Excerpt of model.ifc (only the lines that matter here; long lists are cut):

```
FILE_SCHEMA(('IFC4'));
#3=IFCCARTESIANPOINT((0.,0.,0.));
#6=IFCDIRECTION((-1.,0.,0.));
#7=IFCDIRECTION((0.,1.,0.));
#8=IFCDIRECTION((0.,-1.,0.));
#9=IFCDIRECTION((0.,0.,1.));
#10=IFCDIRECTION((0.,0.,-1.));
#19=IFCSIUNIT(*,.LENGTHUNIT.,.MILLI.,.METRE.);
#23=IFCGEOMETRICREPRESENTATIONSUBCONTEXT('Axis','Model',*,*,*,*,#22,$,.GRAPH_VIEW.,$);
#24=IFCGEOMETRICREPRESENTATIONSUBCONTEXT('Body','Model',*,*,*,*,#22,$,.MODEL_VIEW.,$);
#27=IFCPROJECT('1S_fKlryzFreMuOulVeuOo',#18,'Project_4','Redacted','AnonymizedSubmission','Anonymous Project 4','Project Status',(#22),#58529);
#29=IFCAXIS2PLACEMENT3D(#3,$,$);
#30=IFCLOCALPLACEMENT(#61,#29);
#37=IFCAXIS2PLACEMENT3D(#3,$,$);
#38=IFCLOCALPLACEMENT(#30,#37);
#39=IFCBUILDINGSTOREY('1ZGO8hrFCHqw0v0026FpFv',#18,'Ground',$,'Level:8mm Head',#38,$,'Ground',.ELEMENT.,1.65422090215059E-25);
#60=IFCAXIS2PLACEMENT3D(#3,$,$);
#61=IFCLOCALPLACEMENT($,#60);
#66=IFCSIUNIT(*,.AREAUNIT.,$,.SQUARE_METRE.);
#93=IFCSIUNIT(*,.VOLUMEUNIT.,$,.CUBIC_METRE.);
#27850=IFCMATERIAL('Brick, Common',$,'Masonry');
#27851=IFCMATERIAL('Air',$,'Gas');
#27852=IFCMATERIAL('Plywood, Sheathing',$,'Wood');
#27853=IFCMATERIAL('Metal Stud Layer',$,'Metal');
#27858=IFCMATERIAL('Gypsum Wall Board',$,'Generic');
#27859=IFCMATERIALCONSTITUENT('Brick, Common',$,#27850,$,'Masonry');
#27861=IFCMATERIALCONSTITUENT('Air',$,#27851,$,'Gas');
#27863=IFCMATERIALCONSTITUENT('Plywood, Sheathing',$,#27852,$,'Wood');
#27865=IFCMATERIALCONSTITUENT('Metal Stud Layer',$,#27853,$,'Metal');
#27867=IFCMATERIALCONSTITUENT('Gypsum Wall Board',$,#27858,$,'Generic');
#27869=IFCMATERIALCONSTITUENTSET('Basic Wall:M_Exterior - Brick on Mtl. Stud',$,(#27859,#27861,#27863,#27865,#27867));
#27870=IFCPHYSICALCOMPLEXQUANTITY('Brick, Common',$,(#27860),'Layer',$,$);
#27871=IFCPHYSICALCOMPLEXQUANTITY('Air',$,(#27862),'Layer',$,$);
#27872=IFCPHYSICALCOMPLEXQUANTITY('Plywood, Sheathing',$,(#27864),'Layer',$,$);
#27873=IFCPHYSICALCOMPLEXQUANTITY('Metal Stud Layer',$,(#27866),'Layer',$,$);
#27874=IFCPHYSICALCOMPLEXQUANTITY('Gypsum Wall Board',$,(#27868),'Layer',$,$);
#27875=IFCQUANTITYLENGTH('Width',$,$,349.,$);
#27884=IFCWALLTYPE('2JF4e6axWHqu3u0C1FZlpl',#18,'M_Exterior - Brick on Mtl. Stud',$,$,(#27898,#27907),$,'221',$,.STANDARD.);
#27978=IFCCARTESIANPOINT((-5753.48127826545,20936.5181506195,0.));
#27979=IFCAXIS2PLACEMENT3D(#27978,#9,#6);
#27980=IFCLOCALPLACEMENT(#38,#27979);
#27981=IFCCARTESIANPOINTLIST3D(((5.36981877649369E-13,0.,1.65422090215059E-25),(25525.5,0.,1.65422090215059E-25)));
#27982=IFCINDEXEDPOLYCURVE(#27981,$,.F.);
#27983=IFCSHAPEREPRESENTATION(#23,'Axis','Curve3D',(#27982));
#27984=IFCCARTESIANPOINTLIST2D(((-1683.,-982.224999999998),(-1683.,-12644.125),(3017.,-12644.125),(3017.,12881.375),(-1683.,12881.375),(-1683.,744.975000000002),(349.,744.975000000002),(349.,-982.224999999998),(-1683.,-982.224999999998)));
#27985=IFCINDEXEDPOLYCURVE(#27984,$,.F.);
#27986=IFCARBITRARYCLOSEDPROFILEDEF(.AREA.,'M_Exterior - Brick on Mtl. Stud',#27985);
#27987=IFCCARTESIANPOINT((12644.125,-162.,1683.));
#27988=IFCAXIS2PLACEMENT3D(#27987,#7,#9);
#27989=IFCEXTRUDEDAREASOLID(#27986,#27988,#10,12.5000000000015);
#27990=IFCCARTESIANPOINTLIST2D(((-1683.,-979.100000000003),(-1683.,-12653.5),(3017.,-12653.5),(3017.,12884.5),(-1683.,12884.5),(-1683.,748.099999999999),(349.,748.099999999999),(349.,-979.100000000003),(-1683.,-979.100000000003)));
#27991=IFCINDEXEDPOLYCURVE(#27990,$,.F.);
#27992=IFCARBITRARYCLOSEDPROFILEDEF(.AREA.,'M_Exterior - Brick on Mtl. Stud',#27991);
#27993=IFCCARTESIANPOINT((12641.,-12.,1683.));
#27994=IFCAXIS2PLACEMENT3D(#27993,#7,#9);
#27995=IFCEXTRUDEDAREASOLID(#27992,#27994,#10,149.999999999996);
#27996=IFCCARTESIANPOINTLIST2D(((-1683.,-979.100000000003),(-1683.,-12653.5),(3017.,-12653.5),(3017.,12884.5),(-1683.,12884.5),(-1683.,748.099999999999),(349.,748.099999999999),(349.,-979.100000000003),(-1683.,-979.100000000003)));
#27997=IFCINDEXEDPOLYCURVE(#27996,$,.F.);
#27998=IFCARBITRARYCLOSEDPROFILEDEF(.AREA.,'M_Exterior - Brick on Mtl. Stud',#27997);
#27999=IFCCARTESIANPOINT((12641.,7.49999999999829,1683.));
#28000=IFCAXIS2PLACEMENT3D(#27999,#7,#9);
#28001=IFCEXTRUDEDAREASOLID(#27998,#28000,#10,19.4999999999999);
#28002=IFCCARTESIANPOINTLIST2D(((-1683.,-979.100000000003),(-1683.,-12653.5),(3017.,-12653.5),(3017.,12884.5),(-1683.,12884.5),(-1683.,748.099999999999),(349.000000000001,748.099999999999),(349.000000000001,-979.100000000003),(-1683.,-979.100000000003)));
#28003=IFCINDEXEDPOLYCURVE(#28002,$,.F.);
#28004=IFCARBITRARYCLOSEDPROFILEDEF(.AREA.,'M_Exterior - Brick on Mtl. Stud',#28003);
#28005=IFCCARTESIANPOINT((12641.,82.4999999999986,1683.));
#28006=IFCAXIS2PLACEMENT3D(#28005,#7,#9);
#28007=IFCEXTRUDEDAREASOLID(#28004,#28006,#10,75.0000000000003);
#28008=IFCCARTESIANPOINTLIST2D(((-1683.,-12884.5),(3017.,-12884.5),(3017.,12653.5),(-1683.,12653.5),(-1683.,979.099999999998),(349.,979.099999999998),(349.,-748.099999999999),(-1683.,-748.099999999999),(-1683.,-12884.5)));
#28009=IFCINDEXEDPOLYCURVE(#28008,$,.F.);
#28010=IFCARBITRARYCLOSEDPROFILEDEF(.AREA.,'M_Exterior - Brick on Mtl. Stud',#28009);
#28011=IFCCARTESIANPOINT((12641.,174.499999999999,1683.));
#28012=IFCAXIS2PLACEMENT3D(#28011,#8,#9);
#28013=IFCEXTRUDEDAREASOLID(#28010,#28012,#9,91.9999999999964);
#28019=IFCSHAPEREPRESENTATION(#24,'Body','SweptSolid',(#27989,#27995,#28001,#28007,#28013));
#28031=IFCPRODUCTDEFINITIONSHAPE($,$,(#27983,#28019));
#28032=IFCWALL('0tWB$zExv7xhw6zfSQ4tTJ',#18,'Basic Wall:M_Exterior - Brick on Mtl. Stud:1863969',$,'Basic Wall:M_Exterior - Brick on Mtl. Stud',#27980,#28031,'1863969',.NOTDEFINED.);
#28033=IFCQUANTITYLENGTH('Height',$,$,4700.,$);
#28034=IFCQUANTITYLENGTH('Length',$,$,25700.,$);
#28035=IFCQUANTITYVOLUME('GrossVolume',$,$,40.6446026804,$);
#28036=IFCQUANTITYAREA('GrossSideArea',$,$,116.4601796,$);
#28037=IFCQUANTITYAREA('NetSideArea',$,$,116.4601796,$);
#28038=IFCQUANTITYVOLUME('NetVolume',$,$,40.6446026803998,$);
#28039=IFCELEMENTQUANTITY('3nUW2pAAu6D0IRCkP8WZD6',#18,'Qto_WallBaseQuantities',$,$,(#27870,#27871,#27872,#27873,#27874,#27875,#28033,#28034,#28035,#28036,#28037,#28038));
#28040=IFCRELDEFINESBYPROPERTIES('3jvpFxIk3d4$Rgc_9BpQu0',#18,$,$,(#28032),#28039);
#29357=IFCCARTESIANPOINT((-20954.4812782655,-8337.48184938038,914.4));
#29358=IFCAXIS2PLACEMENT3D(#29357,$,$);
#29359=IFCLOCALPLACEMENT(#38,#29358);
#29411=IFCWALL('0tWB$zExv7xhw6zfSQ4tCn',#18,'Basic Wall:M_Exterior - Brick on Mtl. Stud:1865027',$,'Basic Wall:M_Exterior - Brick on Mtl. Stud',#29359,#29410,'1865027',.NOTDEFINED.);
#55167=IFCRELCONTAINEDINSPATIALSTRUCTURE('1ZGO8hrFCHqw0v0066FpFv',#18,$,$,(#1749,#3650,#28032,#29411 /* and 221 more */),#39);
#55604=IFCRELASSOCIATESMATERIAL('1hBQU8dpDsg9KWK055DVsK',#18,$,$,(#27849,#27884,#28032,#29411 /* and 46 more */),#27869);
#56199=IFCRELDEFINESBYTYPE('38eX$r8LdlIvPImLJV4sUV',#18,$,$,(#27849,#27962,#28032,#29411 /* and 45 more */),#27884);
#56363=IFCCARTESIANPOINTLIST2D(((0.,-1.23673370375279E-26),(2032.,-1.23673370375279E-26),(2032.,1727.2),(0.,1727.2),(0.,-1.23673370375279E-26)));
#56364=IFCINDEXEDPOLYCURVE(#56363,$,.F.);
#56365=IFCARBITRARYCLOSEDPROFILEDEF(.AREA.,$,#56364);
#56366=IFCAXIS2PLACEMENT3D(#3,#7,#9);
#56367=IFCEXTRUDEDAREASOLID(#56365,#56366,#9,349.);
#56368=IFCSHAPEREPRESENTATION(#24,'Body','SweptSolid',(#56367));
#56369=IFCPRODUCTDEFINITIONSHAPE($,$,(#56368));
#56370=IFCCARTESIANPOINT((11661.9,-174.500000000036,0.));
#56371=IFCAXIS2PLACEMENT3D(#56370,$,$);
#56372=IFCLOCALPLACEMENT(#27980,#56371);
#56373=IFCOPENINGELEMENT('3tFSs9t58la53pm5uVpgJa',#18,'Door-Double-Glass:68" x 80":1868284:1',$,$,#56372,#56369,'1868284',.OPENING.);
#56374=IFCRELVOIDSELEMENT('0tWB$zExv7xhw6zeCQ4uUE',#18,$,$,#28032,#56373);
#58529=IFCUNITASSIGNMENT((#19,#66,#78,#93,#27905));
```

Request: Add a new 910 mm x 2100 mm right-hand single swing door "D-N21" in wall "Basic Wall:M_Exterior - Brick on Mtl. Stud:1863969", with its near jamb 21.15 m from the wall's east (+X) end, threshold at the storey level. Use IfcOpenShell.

```python
import numpy as np
import ifcopenshell
import ifcopenshell.api.feature
import ifcopenshell.api.geometry
import ifcopenshell.api.pset
import ifcopenshell.api.root
import ifcopenshell.api.spatial
import ifcopenshell.geom
import ifcopenshell.util.element
import ifcopenshell.util.placement
import ifcopenshell.util.representation
import ifcopenshell.util.shape
import ifcopenshell.util.unit

model = ifcopenshell.open("model.ifc")
unit_scale = ifcopenshell.util.unit.calculate_unit_scale(model)
area_scale = ifcopenshell.util.unit.calculate_unit_scale(model, "AREAUNIT")
volume_scale = ifcopenshell.util.unit.calculate_unit_scale(model, "VOLUMEUNIT")
settings = ifcopenshell.geom.settings()


def volume(element):
    """Net volume in cubic metres, openings subtracted."""
    shape = ifcopenshell.geom.create_shape(settings, element)
    return ifcopenshell.util.shape.get_volume(shape.geometry)


wall = model.by_id(28032)
storey = ifcopenshell.util.element.get_container(wall, ifc_class="IfcBuildingStorey")
context = ifcopenshell.util.representation.get_context(model, "Model", "Body", "MODEL_VIEW")
before = volume(wall)

width, height, from_end, sill = 0.91, 2.1, 21.15, 0.0  # metres

# The wall runs along its own X axis, and the end named is its -X end.
wall_shape = ifcopenshell.geom.create_shape(settings, wall)
x, y, z = ifcopenshell.util.shape.get_vertices(wall_shape.geometry).T
start = x.min() + from_end
face, thickness = float(y.min()), float(y.max() - y.min())
wall_matrix = ifcopenshell.util.placement.get_local_placement(wall.ObjectPlacement)
level = ifcopenshell.util.placement.get_local_placement(storey.ObjectPlacement)[2, 3]


def in_wall(x, y):
    """Placement at x, y metres in the wall's axes, at sill height."""
    matrix = wall_matrix.copy()
    matrix[:, 3] = wall_matrix @ np.array([x / unit_scale, y / unit_scale, 0.0, 1.0])
    matrix[2, 3] = level + sill / unit_scale
    return matrix


# Opening: a box that overshoots both wall faces by 50 mm.
opening = ifcopenshell.api.root.create_entity(model, ifc_class="IfcOpeningElement", predefined_type="OPENING")
box = ifcopenshell.api.geometry.add_wall_representation(
    model, context=context, length=width, height=height, thickness=thickness + 0.1
)
ifcopenshell.api.geometry.assign_representation(model, product=opening, representation=box)
ifcopenshell.api.geometry.edit_object_placement(model, product=opening, matrix=in_wall(start, face - 0.05), is_si=False)
ifcopenshell.api.feature.add_feature(model, feature=opening, element=wall)

door = ifcopenshell.api.root.create_entity(model, ifc_class="IfcDoor", name="D-N21", predefined_type="DOOR")
door.OverallWidth, door.OverallHeight = width / unit_scale, height / unit_scale
door.OperationType = "SINGLE_SWING_RIGHT"
body = ifcopenshell.api.geometry.add_door_representation(
    model,
    context=context,
    overall_width=door.OverallWidth,
    overall_height=door.OverallHeight,
    operation_type="SINGLE_SWING_RIGHT",
    lining_properties={"LiningDepth": thickness / unit_scale, "ThresholdDepth": thickness / unit_scale},
)
ifcopenshell.api.geometry.assign_representation(model, product=door, representation=body)
ifcopenshell.api.spatial.assign_container(model, products=[door], relating_structure=storey)
ifcopenshell.api.feature.add_filling(model, opening=opening, element=door)

# The lining spans the wall, so the door starts at the wall face.
ifcopenshell.api.geometry.edit_object_placement(model, product=door, matrix=in_wall(start, face), is_si=False)

after = volume(wall)

# Update the wall's stored quantities.
qto = model.by_id(ifcopenshell.util.element.get_pset(wall, "Qto_WallBaseQuantities", should_inherit=False)["id"])
ifcopenshell.api.pset.edit_qto(model, qto=qto, properties={
    "NetSideArea": after / thickness / area_scale,
    "NetVolume": after / volume_scale,
})

print(f"wall volume {before:.3f} -> {after:.3f} m3")

model.write("model_edited.ifc")
```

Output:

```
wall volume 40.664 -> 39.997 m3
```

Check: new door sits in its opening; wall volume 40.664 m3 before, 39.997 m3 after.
